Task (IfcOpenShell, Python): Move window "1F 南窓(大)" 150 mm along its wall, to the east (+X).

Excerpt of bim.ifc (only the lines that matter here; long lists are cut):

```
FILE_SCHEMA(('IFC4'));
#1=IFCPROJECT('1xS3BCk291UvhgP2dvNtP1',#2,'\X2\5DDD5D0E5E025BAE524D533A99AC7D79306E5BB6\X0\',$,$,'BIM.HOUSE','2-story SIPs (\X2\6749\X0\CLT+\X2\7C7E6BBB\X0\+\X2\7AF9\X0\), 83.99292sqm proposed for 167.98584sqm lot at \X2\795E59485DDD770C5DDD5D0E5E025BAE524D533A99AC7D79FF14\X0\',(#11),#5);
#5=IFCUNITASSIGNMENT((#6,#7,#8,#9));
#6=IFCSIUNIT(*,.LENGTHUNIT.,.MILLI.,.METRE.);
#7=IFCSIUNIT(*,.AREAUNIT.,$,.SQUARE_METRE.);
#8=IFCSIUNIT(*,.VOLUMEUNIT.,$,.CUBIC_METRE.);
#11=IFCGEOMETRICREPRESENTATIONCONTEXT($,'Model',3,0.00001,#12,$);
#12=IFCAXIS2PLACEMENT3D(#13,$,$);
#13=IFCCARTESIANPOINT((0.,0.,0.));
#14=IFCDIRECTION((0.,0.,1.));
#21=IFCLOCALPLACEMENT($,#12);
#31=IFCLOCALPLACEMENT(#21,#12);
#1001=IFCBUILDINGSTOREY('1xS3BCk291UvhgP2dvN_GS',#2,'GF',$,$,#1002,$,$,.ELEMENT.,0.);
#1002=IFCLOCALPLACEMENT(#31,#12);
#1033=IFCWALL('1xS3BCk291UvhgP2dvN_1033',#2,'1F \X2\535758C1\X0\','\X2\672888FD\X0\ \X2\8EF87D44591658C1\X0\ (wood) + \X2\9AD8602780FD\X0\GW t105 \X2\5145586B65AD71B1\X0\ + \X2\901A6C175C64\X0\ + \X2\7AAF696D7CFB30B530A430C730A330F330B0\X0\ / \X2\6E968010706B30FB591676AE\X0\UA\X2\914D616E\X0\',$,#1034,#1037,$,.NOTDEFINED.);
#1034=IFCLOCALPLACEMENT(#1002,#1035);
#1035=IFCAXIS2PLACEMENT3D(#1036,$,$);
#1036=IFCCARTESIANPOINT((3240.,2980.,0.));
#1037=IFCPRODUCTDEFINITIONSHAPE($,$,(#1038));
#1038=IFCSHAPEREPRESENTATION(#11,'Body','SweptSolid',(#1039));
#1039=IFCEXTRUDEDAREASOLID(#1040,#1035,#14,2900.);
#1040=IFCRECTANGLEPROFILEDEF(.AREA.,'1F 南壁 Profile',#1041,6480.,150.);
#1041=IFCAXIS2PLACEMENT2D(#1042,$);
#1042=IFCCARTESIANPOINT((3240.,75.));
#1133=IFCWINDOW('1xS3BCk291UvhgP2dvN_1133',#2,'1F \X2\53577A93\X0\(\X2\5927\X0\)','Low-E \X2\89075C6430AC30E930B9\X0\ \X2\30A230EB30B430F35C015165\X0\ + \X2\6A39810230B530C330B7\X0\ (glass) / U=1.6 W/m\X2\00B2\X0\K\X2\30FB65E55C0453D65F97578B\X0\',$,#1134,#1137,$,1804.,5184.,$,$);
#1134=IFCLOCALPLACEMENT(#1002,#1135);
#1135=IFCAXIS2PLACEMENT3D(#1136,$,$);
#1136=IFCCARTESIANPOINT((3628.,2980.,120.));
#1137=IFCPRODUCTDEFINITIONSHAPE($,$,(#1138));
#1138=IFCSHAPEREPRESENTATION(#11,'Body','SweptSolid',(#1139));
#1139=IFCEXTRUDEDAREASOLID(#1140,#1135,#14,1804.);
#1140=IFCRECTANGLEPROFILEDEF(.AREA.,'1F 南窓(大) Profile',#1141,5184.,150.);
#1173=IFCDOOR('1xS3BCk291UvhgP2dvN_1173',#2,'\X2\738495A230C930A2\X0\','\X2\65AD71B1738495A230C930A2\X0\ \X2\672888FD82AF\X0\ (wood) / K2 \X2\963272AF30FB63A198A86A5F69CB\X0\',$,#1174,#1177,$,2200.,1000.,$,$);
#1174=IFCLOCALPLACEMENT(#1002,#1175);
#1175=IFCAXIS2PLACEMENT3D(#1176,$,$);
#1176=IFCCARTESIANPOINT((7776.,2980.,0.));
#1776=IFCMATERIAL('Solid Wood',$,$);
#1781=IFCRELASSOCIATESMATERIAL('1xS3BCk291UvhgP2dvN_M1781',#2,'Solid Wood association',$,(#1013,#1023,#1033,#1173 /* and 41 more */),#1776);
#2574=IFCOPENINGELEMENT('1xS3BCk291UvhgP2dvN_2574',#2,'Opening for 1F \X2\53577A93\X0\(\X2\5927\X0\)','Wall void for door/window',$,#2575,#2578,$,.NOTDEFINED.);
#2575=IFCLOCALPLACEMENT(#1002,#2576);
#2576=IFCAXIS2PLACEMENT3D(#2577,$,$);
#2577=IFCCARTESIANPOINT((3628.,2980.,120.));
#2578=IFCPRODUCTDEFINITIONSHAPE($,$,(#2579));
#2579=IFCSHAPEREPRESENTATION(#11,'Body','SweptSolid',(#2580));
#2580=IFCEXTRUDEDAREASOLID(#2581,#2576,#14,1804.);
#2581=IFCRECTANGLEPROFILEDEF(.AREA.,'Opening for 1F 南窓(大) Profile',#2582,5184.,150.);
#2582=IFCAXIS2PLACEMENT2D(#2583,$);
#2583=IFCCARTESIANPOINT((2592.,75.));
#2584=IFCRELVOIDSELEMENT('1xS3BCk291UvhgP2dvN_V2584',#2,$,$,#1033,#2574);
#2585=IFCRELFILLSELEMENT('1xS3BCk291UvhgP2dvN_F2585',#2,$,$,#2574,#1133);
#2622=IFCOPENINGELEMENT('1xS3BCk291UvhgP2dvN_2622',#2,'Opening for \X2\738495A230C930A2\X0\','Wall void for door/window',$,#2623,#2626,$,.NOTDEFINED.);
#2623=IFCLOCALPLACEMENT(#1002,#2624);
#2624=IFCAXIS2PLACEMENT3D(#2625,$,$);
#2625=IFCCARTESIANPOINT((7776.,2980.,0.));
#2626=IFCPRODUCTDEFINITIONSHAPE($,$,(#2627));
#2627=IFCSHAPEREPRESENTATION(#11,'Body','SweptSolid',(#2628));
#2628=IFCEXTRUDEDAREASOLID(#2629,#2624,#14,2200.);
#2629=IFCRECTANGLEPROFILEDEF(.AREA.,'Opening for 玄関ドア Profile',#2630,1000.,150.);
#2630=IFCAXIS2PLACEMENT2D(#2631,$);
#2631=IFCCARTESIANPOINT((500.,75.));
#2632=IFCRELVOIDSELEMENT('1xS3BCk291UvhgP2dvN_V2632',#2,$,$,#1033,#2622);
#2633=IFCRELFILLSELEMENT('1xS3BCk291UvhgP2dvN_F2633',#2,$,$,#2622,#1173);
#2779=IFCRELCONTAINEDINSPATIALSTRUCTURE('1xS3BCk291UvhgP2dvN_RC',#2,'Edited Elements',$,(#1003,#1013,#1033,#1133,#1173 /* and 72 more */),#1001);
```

```python
import ifcopenshell
import ifcopenshell.api.geometry
import ifcopenshell.util.placement

model = ifcopenshell.open("bim.ifc")

window = model.by_id(1133)
opening = window.FillsVoids[0].RelatingOpeningElement
wall = opening.VoidsElements[0].RelatingBuildingElement

wall_matrix = ifcopenshell.util.placement.get_local_placement(wall.ObjectPlacement)
shift = wall_matrix[:3, 0] * 150.0
before = ifcopenshell.util.placement.get_local_placement(window.ObjectPlacement)[:3, 3].copy()

# The window is not placed relative to its opening, so move both.
for product in (opening, window):
    matrix = ifcopenshell.util.placement.get_local_placement(product.ObjectPlacement)
    matrix[:3, 3] += shift
    ifcopenshell.api.geometry.edit_object_placement(model, product=product, matrix=matrix, is_si=False)

after = ifcopenshell.util.placement.get_local_placement(window.ObjectPlacement)[:3, 3]
print("window moved by", (after - before).round(3) + 0.0)

model.write("bim-out.ifc")
```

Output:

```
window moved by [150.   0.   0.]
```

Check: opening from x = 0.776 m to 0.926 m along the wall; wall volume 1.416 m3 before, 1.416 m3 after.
